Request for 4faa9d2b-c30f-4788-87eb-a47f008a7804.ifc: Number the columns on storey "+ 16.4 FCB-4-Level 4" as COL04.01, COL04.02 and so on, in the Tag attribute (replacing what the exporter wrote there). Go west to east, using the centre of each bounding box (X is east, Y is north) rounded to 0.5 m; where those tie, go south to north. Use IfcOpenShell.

First a look at what the model holds.

```python
import ifcopenshell
import ifcopenshell.util.element
import ifcopenshell.util.placement

model = ifcopenshell.open("4faa9d2b-c30f-4788-87eb-a47f008a7804.ifc")
print(model.schema)
storey = next(s for s in model.by_type("IfcBuildingStorey") if s.Name == "+ 16.4 FCB-4-Level 4")
columns = [e for e in ifcopenshell.util.element.get_decomposition(storey) if e.is_a("IfcColumn")]
for e in sorted(columns, key=lambda e: e.id()):
    origin = ifcopenshell.util.placement.get_local_placement(e.ObjectPlacement)[:3, 3]
    print(e.id(), e.Tag, e.Name, origin.round(2) + 0.0, sep=" | ")
```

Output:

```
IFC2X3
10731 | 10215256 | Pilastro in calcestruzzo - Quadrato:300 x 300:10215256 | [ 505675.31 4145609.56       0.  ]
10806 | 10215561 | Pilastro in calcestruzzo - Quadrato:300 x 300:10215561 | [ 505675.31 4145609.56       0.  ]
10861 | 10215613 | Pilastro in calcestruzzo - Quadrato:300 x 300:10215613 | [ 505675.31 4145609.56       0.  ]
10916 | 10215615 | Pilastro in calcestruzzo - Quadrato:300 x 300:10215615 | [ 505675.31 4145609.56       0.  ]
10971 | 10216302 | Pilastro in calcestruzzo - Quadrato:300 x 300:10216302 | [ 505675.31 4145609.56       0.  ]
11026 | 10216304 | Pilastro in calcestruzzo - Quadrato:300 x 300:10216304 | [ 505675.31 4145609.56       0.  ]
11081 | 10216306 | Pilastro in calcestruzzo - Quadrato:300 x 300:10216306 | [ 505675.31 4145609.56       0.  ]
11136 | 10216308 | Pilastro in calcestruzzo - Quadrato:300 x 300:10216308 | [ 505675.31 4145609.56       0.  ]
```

```python
import ifcopenshell
import ifcopenshell.geom
import ifcopenshell.util.element
import ifcopenshell.util.shape

model = ifcopenshell.open("4faa9d2b-c30f-4788-87eb-a47f008a7804.ifc")
settings = ifcopenshell.geom.settings()
settings.set("use-world-coords", True)


def centre(element):
    shape = ifcopenshell.geom.create_shape(settings, element)
    return ifcopenshell.util.shape.get_bbox_centroid(shape.geometry)


storey = next(s for s in model.by_type("IfcBuildingStorey") if s.Name == "+ 16.4 FCB-4-Level 4")
columns = [e for e in ifcopenshell.util.element.get_decomposition(storey) if e.is_a("IfcColumn")]

# Insertion points can sit at a corner or the storey origin, so sort by the geometry (in metres).
centres = {e: centre(e) for e in columns}
columns.sort(key=lambda e: (round(centres[e][0] / 0.5), centres[e][1]))

for i, e in enumerate(columns, start=1):
    number = f"COL04.{i:02d}"
    e.Tag = number
    print(e.id(), number)

model.write("4faa9d2b-c30f-4788-87eb-a47f008a7804_v2.ifc")
```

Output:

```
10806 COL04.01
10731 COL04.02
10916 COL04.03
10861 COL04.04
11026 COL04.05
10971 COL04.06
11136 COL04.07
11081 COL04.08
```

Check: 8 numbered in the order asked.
